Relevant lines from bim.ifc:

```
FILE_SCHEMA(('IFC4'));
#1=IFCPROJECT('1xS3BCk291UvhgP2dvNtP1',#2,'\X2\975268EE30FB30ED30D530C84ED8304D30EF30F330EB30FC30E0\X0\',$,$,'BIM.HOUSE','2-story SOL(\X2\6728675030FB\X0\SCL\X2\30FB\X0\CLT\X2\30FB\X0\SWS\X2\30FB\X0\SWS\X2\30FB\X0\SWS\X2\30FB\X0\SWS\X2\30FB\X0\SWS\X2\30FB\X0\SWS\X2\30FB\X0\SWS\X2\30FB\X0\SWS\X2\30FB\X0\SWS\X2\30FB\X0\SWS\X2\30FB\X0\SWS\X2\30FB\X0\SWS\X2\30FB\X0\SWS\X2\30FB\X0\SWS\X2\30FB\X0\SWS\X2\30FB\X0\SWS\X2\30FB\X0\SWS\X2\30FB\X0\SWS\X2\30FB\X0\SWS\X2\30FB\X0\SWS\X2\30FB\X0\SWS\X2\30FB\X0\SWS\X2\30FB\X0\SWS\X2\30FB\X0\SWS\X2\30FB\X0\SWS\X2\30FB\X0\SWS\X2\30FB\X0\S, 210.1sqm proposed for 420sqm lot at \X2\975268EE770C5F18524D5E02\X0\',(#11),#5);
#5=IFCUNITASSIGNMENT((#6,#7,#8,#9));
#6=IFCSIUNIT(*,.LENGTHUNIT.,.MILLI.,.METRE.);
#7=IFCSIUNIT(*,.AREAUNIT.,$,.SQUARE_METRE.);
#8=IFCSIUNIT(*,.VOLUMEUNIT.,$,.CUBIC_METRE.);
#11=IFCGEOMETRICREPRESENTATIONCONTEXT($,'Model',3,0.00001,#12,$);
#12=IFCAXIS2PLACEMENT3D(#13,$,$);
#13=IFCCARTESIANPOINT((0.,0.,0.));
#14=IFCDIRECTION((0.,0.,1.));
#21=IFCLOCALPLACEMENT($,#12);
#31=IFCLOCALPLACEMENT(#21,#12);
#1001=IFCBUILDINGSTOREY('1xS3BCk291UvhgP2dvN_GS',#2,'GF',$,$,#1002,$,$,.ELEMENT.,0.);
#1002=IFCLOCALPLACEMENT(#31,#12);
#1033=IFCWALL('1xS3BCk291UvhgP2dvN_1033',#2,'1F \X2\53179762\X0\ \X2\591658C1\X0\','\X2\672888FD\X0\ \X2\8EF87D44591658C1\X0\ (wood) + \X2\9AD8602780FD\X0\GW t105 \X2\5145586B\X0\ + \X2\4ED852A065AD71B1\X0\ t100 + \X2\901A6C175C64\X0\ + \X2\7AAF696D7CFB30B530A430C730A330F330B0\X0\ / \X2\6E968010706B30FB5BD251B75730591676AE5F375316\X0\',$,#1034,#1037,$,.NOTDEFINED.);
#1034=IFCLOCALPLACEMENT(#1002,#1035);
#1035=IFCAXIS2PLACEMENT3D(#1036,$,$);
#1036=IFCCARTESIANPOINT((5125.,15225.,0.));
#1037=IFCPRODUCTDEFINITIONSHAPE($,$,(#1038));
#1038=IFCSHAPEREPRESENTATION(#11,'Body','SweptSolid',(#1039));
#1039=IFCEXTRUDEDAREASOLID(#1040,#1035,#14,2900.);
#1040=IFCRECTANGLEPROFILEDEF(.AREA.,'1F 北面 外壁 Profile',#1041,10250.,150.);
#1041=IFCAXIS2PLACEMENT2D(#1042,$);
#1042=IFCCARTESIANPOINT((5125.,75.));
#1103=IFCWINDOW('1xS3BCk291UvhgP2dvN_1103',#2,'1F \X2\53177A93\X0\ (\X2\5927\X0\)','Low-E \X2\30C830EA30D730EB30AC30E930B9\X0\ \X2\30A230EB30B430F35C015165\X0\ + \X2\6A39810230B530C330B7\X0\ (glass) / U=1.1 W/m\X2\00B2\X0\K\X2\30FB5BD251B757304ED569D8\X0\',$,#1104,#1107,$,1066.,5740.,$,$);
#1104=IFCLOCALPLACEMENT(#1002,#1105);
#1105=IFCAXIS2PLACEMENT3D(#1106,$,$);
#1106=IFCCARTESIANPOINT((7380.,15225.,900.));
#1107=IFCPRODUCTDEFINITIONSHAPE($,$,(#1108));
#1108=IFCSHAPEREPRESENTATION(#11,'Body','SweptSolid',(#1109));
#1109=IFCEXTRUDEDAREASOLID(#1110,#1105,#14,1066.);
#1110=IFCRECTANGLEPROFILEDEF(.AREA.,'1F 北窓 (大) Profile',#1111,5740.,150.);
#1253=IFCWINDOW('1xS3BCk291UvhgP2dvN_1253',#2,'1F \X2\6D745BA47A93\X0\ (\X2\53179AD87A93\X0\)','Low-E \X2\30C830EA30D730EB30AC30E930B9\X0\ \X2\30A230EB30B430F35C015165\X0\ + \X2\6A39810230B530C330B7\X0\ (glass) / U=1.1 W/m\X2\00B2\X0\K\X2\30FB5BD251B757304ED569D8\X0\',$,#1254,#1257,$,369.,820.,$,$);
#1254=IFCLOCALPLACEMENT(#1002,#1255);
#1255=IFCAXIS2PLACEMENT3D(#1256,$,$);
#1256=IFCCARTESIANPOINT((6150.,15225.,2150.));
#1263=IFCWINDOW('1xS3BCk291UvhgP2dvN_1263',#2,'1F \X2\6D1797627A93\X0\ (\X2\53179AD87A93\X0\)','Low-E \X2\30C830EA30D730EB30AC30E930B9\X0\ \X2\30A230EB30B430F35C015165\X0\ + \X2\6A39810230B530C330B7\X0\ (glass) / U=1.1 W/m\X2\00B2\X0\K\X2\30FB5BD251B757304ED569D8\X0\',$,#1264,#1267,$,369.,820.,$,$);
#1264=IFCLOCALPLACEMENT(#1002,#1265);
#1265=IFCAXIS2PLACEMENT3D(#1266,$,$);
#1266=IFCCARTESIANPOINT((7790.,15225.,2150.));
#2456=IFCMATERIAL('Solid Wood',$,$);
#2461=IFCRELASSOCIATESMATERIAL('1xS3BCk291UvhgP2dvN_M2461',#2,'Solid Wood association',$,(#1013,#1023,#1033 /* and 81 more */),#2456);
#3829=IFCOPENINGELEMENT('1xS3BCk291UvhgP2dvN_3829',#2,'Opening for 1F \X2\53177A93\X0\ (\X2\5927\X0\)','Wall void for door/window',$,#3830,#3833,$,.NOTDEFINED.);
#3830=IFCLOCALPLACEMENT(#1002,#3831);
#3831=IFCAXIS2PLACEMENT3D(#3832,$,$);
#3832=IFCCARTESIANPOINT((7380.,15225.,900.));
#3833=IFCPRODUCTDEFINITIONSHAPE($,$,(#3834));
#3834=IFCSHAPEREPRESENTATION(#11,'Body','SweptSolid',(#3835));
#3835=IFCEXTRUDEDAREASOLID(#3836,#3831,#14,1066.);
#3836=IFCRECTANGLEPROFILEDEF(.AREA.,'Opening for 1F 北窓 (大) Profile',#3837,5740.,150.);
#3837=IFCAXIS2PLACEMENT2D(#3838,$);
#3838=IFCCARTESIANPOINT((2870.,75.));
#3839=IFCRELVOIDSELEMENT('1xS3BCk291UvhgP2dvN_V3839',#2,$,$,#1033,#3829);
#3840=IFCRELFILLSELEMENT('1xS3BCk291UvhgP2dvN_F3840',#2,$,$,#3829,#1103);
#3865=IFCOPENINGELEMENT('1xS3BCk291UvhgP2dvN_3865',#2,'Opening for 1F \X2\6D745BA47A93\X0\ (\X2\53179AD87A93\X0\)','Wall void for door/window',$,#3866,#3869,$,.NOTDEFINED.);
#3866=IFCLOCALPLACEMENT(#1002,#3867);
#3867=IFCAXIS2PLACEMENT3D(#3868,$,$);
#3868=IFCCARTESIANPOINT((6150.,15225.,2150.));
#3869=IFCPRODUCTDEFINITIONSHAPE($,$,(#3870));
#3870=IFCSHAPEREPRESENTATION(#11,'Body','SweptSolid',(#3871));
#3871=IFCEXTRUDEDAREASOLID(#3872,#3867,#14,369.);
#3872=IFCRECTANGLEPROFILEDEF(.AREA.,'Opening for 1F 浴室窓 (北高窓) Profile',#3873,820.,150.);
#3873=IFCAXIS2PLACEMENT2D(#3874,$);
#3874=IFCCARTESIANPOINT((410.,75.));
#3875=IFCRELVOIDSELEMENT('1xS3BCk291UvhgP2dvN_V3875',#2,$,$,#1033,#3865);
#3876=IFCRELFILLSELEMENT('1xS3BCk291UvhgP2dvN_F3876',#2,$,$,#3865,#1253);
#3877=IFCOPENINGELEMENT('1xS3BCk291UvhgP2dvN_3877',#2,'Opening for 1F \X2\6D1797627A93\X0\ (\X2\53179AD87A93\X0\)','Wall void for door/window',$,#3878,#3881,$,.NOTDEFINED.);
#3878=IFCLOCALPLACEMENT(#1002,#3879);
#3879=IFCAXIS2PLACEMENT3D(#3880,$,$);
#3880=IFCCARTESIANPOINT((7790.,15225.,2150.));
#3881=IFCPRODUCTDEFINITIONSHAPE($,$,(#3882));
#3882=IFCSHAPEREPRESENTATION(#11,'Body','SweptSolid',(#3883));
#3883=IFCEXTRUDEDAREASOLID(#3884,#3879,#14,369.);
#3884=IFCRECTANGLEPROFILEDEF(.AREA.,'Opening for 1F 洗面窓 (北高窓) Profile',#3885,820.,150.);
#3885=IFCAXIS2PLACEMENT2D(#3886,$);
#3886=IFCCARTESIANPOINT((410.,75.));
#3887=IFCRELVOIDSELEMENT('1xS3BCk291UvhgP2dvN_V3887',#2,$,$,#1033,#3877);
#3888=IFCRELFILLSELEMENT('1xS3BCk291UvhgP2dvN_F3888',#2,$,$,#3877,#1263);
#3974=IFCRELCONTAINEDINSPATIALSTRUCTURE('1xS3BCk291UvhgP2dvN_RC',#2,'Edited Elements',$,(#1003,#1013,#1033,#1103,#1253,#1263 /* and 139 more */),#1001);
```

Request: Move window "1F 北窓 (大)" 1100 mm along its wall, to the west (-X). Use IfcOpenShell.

```python
import ifcopenshell
import ifcopenshell.api.geometry
import ifcopenshell.util.placement

model = ifcopenshell.open("bim.ifc")

window = model.by_guid("1xS3BCk291UvhgP2dvN_1103")
opening = window.FillsVoids[0].RelatingOpeningElement
wall = opening.VoidsElements[0].RelatingBuildingElement

wall_matrix = ifcopenshell.util.placement.get_local_placement(wall.ObjectPlacement)
shift = wall_matrix[:3, 0] * -1100.0
before = ifcopenshell.util.placement.get_local_placement(window.ObjectPlacement)[:3, 3].copy()

# The window is not placed relative to its opening, so move both.
for product in (opening, window):
    matrix = ifcopenshell.util.placement.get_local_placement(product.ObjectPlacement)
    matrix[:3, 3] += shift
    ifcopenshell.api.geometry.edit_object_placement(model, product=product, matrix=matrix, is_si=False)

after = ifcopenshell.util.placement.get_local_placement(window.ObjectPlacement)[:3, 3]
print("window moved by", (after - before).round(3) + 0.0)

model.write("bim_v2.ifc")
```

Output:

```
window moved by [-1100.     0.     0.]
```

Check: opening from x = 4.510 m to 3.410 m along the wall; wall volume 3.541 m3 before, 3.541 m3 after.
